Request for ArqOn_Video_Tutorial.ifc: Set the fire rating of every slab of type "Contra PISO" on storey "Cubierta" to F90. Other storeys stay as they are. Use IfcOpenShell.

First a look at what the model holds.

```python
import ifcopenshell
import ifcopenshell.util.element

model = ifcopenshell.open("ArqOn_Video_Tutorial.ifc")
print(model.schema)
storey = next(s for s in model.by_type("IfcBuildingStorey") if s.Name == "Cubierta")
slabs = [e for e in ifcopenshell.util.element.get_decomposition(storey) if e.is_a("IfcSlab")]
seen = {}
for e in slabs:
    element_type = ifcopenshell.util.element.get_type(e)
    key = (element_type.Name if element_type != e and element_type else None, ifcopenshell.util.element.get_pset(e, "Pset_SlabCommon", "FireRating"))
    seen[key] = seen.get(key, 0) + 1
for (name, value), count in sorted(seen.items(), key=str):
    print(count, "x", name, "|", value)
```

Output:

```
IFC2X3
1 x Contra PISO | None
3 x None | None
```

```python
import ifcopenshell
import ifcopenshell.api.pset
import ifcopenshell.util.element

model = ifcopenshell.open("ArqOn_Video_Tutorial.ifc")

storey = next(s for s in model.by_type("IfcBuildingStorey") if s.Name == "Cubierta")
slabs = [e for e in ifcopenshell.util.element.get_decomposition(storey) if e.is_a("IfcSlab")]

count = 0
for e in slabs:
    element_type = ifcopenshell.util.element.get_type(e)
    if element_type in (None, e) or element_type.Name != "Contra PISO":
        continue
    # add_pset returns the element's existing set when there is one.
    pset = ifcopenshell.api.pset.add_pset(model, product=e, name="Pset_SlabCommon")
    ifcopenshell.api.pset.edit_pset(model, pset=pset, properties={"FireRating": "F90"})
    count += 1

print(count, "slabs updated")

model.write("ArqOn_Video_Tutorial_updated.ifc")
```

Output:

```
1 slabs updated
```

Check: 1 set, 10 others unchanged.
